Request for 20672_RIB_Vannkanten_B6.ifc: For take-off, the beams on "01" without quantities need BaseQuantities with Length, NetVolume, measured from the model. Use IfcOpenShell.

First a look at what the model holds.

```python
import ifcopenshell
import ifcopenshell.util.element
import ifcopenshell.util.unit

model = ifcopenshell.open("20672_RIB_Vannkanten_B6.ifc")
print(model.schema)
for unit_type in ("LENGTHUNIT", "AREAUNIT", "VOLUMEUNIT"):
    print(unit_type, ifcopenshell.util.unit.calculate_unit_scale(model, unit_type))
storey = next(s for s in model.by_type("IfcBuildingStorey") if s.Name == "01")
beams = [e for e in ifcopenshell.util.element.get_decomposition(storey) if e.is_a("IfcBeam")]
for e in sorted(beams, key=lambda e: e.id()):
    print(e.id(), e.is_a(), e.Name, list(ifcopenshell.util.element.get_psets(e, qtos_only=True)), sep=" | ")
```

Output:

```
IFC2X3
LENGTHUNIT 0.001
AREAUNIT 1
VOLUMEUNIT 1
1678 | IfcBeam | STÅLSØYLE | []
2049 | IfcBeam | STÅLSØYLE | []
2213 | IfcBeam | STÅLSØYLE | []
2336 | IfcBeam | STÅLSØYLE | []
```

```python
import ifcopenshell
import ifcopenshell.api.pset
import ifcopenshell.geom
import ifcopenshell.util.element
import ifcopenshell.util.shape
import ifcopenshell.util.unit

model = ifcopenshell.open("20672_RIB_Vannkanten_B6.ifc")
unit_scale = ifcopenshell.util.unit.calculate_unit_scale(model)
volume_scale = ifcopenshell.util.unit.calculate_unit_scale(model, "VOLUMEUNIT")
settings = ifcopenshell.geom.settings()

storey = next(s for s in model.by_type("IfcBuildingStorey") if s.Name == "01")
beams = [e for e in ifcopenshell.util.element.get_decomposition(storey) if e.is_a("IfcBeam")]

for e in sorted(beams, key=lambda e: e.id()):
    if ifcopenshell.util.element.get_psets(e, qtos_only=True, should_inherit=False):
        continue
    # Geometry comes back in metres, in the element's own axes.
    shape = ifcopenshell.geom.create_shape(settings, e)
    values = {
        "Length": ifcopenshell.util.shape.get_max_xyz(shape.geometry) / unit_scale,
        "NetVolume": ifcopenshell.util.shape.get_volume(shape.geometry) / volume_scale,
    }
    qto = ifcopenshell.api.pset.add_qto(model, product=e, name="BaseQuantities")
    ifcopenshell.api.pset.edit_qto(model, qto=qto, properties=values)
    print(e.id(), {k: round(v, 3) for k, v in values.items()})

model.write("20672_RIB_Vannkanten_B6_edited.ifc")
```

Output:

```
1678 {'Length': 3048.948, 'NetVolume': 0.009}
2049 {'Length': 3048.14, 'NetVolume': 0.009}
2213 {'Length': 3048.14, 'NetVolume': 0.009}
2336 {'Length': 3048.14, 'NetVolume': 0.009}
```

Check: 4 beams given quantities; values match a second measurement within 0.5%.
